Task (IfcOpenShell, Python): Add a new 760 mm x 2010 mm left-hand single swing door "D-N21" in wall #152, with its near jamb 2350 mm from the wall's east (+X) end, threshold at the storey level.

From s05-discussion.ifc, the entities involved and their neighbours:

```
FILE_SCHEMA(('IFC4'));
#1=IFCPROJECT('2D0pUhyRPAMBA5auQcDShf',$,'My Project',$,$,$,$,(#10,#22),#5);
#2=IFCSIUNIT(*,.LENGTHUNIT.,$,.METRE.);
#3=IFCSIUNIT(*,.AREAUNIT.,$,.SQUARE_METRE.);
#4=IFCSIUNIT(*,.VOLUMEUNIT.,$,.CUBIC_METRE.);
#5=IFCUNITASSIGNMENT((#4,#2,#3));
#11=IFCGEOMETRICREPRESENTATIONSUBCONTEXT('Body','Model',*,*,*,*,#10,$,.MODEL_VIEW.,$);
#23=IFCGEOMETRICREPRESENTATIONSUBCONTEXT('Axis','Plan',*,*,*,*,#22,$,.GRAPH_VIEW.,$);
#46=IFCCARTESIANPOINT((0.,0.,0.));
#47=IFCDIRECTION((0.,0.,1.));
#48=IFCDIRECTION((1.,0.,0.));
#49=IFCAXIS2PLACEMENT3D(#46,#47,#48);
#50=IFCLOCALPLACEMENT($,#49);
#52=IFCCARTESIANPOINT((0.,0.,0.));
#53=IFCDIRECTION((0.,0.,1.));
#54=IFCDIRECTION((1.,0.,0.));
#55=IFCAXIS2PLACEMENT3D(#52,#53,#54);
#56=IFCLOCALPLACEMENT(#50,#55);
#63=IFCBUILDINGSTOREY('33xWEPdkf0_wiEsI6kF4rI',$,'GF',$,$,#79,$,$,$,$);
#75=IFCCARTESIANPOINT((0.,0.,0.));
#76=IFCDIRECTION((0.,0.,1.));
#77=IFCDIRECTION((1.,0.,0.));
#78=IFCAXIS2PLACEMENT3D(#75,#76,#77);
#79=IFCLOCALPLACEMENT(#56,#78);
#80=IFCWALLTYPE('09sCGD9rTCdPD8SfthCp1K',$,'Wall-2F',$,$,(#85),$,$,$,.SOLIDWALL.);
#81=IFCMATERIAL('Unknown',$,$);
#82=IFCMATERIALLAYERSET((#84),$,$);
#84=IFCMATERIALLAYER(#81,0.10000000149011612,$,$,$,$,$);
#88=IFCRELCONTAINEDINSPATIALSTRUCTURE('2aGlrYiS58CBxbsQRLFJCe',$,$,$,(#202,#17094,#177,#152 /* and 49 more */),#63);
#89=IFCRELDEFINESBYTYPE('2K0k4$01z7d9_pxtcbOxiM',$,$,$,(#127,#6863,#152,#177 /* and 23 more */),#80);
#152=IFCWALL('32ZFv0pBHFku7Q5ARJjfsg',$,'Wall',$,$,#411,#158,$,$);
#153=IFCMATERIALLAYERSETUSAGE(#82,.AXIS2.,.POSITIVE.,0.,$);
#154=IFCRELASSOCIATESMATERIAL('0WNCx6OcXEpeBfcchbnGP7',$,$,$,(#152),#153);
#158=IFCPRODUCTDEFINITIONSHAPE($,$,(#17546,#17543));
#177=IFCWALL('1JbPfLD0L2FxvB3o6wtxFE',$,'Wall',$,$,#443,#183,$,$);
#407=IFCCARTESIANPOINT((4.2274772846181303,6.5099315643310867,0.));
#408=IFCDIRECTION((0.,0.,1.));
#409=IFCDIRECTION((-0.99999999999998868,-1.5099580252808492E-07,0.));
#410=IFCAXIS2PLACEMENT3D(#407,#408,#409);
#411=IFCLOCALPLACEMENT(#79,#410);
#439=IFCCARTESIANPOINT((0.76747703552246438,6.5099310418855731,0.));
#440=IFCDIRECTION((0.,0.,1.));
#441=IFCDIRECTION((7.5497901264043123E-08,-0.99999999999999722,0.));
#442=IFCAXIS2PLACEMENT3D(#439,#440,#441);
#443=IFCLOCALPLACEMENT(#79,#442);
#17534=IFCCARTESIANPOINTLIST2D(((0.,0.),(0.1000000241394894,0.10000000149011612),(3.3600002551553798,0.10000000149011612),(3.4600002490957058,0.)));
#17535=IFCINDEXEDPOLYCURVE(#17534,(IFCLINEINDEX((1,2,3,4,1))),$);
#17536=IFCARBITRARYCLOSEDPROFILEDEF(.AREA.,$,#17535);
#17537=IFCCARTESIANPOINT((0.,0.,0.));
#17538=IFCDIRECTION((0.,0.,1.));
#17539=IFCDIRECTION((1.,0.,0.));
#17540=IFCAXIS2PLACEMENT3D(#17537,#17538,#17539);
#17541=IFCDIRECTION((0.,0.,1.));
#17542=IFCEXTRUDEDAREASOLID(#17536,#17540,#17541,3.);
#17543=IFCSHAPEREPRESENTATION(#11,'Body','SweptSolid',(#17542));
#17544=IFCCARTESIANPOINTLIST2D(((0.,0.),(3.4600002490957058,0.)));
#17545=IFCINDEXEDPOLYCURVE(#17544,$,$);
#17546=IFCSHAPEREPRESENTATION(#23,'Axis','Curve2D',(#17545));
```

```python
import numpy as np
import ifcopenshell
import ifcopenshell.api.feature
import ifcopenshell.api.geometry
import ifcopenshell.api.root
import ifcopenshell.api.spatial
import ifcopenshell.geom
import ifcopenshell.util.element
import ifcopenshell.util.placement
import ifcopenshell.util.representation
import ifcopenshell.util.shape
import ifcopenshell.util.unit

model = ifcopenshell.open("s05-discussion.ifc")
unit_scale = ifcopenshell.util.unit.calculate_unit_scale(model)
settings = ifcopenshell.geom.settings()


def volume(element):
    """Net volume in cubic metres, openings subtracted."""
    shape = ifcopenshell.geom.create_shape(settings, element)
    return ifcopenshell.util.shape.get_volume(shape.geometry)


wall = model.by_guid("32ZFv0pBHFku7Q5ARJjfsg")
storey = ifcopenshell.util.element.get_container(wall, ifc_class="IfcBuildingStorey")
context = ifcopenshell.util.representation.get_context(model, "Model", "Body", "MODEL_VIEW")
before = volume(wall)

width, height, from_end, sill = 0.76, 2.01, 2.35, 0.0  # metres

# The wall runs along its own X axis, and the end named is its -X end.
wall_shape = ifcopenshell.geom.create_shape(settings, wall)
x, y, z = ifcopenshell.util.shape.get_vertices(wall_shape.geometry).T
start = x.min() + from_end
face, thickness = float(y.min()), float(y.max() - y.min())
wall_matrix = ifcopenshell.util.placement.get_local_placement(wall.ObjectPlacement)
level = ifcopenshell.util.placement.get_local_placement(storey.ObjectPlacement)[2, 3]


def in_wall(x, y):
    """Placement at x, y metres in the wall's axes, at sill height."""
    matrix = wall_matrix.copy()
    matrix[:, 3] = wall_matrix @ np.array([x / unit_scale, y / unit_scale, 0.0, 1.0])
    matrix[2, 3] = level + sill / unit_scale
    return matrix


# Opening: a box that overshoots both wall faces by 50 mm.
opening = ifcopenshell.api.root.create_entity(model, ifc_class="IfcOpeningElement", predefined_type="OPENING")
box = ifcopenshell.api.geometry.add_wall_representation(
    model, context=context, length=width, height=height, thickness=thickness + 0.1
)
ifcopenshell.api.geometry.assign_representation(model, product=opening, representation=box)
ifcopenshell.api.geometry.edit_object_placement(model, product=opening, matrix=in_wall(start, face - 0.05), is_si=False)
ifcopenshell.api.feature.add_feature(model, feature=opening, element=wall)

door = ifcopenshell.api.root.create_entity(model, ifc_class="IfcDoor", name="D-N21", predefined_type="DOOR")
door.OverallWidth, door.OverallHeight = width / unit_scale, height / unit_scale
door.OperationType = "SINGLE_SWING_LEFT"
body = ifcopenshell.api.geometry.add_door_representation(
    model,
    context=context,
    overall_width=door.OverallWidth,
    overall_height=door.OverallHeight,
    operation_type="SINGLE_SWING_LEFT",
    lining_properties={"LiningDepth": thickness / unit_scale, "ThresholdDepth": thickness / unit_scale},
)
ifcopenshell.api.geometry.assign_representation(model, product=door, representation=body)
ifcopenshell.api.spatial.assign_container(model, products=[door], relating_structure=storey)
ifcopenshell.api.feature.add_filling(model, opening=opening, element=door)

# The lining spans the wall, so the door starts at the wall face.
ifcopenshell.api.geometry.edit_object_placement(model, product=door, matrix=in_wall(start, face), is_si=False)

after = volume(wall)

print(f"wall volume {before:.3f} -> {after:.3f} m3")

model.write("s05-discussion_updated.ifc")
```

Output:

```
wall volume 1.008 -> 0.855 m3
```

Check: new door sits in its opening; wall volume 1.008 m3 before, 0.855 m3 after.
